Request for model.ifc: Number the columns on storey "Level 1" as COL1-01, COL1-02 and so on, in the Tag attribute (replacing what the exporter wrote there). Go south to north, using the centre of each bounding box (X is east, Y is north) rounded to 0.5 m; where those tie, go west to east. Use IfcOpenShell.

First a look at what the model holds.

```python
import ifcopenshell
import ifcopenshell.util.element
import ifcopenshell.util.placement

model = ifcopenshell.open("model.ifc")
print(model.schema)
storey = next(s for s in model.by_type("IfcBuildingStorey") if s.Name == "Level 1")
columns = [e for e in ifcopenshell.util.element.get_decomposition(storey) if e.is_a("IfcColumn")]
for e in sorted(columns, key=lambda e: e.id()):
    origin = ifcopenshell.util.placement.get_local_placement(e.ObjectPlacement)[:3, 3]
    print(e.id(), e.Tag, e.Name, origin.round(2) + 0.0, sep=" | ")
```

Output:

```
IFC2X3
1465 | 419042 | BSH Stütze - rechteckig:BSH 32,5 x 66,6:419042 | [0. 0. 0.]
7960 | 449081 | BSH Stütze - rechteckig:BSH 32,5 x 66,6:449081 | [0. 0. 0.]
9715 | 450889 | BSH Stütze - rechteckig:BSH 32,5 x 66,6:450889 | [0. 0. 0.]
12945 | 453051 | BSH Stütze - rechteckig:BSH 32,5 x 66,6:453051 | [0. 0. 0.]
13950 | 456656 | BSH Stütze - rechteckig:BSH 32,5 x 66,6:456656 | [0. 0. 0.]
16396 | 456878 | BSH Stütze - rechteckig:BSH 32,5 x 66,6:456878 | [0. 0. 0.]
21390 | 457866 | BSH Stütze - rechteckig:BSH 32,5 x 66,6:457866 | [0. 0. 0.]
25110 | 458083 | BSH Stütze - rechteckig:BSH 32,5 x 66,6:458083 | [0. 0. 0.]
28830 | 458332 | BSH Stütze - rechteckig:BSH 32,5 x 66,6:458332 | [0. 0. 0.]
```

```python
import ifcopenshell
import ifcopenshell.geom
import ifcopenshell.util.element
import ifcopenshell.util.shape

model = ifcopenshell.open("model.ifc")
settings = ifcopenshell.geom.settings()
settings.set("use-world-coords", True)


def centre(element):
    shape = ifcopenshell.geom.create_shape(settings, element)
    return ifcopenshell.util.shape.get_bbox_centroid(shape.geometry)


storey = next(s for s in model.by_type("IfcBuildingStorey") if s.Name == "Level 1")
columns = [e for e in ifcopenshell.util.element.get_decomposition(storey) if e.is_a("IfcColumn")]

# Insertion points can sit at a corner or the storey origin, so sort by the geometry (in metres).
centres = {e: centre(e) for e in columns}
columns.sort(key=lambda e: (round(centres[e][1] / 0.5), centres[e][0]))

for i, e in enumerate(columns, start=1):
    number = f"COL1-{i:02d}"
    e.Tag = number
    print(e.id(), number)

model.write("model_v2.ifc")
```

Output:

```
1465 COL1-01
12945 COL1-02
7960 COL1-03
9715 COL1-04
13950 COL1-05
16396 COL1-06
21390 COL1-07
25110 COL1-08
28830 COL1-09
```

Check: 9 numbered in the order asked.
